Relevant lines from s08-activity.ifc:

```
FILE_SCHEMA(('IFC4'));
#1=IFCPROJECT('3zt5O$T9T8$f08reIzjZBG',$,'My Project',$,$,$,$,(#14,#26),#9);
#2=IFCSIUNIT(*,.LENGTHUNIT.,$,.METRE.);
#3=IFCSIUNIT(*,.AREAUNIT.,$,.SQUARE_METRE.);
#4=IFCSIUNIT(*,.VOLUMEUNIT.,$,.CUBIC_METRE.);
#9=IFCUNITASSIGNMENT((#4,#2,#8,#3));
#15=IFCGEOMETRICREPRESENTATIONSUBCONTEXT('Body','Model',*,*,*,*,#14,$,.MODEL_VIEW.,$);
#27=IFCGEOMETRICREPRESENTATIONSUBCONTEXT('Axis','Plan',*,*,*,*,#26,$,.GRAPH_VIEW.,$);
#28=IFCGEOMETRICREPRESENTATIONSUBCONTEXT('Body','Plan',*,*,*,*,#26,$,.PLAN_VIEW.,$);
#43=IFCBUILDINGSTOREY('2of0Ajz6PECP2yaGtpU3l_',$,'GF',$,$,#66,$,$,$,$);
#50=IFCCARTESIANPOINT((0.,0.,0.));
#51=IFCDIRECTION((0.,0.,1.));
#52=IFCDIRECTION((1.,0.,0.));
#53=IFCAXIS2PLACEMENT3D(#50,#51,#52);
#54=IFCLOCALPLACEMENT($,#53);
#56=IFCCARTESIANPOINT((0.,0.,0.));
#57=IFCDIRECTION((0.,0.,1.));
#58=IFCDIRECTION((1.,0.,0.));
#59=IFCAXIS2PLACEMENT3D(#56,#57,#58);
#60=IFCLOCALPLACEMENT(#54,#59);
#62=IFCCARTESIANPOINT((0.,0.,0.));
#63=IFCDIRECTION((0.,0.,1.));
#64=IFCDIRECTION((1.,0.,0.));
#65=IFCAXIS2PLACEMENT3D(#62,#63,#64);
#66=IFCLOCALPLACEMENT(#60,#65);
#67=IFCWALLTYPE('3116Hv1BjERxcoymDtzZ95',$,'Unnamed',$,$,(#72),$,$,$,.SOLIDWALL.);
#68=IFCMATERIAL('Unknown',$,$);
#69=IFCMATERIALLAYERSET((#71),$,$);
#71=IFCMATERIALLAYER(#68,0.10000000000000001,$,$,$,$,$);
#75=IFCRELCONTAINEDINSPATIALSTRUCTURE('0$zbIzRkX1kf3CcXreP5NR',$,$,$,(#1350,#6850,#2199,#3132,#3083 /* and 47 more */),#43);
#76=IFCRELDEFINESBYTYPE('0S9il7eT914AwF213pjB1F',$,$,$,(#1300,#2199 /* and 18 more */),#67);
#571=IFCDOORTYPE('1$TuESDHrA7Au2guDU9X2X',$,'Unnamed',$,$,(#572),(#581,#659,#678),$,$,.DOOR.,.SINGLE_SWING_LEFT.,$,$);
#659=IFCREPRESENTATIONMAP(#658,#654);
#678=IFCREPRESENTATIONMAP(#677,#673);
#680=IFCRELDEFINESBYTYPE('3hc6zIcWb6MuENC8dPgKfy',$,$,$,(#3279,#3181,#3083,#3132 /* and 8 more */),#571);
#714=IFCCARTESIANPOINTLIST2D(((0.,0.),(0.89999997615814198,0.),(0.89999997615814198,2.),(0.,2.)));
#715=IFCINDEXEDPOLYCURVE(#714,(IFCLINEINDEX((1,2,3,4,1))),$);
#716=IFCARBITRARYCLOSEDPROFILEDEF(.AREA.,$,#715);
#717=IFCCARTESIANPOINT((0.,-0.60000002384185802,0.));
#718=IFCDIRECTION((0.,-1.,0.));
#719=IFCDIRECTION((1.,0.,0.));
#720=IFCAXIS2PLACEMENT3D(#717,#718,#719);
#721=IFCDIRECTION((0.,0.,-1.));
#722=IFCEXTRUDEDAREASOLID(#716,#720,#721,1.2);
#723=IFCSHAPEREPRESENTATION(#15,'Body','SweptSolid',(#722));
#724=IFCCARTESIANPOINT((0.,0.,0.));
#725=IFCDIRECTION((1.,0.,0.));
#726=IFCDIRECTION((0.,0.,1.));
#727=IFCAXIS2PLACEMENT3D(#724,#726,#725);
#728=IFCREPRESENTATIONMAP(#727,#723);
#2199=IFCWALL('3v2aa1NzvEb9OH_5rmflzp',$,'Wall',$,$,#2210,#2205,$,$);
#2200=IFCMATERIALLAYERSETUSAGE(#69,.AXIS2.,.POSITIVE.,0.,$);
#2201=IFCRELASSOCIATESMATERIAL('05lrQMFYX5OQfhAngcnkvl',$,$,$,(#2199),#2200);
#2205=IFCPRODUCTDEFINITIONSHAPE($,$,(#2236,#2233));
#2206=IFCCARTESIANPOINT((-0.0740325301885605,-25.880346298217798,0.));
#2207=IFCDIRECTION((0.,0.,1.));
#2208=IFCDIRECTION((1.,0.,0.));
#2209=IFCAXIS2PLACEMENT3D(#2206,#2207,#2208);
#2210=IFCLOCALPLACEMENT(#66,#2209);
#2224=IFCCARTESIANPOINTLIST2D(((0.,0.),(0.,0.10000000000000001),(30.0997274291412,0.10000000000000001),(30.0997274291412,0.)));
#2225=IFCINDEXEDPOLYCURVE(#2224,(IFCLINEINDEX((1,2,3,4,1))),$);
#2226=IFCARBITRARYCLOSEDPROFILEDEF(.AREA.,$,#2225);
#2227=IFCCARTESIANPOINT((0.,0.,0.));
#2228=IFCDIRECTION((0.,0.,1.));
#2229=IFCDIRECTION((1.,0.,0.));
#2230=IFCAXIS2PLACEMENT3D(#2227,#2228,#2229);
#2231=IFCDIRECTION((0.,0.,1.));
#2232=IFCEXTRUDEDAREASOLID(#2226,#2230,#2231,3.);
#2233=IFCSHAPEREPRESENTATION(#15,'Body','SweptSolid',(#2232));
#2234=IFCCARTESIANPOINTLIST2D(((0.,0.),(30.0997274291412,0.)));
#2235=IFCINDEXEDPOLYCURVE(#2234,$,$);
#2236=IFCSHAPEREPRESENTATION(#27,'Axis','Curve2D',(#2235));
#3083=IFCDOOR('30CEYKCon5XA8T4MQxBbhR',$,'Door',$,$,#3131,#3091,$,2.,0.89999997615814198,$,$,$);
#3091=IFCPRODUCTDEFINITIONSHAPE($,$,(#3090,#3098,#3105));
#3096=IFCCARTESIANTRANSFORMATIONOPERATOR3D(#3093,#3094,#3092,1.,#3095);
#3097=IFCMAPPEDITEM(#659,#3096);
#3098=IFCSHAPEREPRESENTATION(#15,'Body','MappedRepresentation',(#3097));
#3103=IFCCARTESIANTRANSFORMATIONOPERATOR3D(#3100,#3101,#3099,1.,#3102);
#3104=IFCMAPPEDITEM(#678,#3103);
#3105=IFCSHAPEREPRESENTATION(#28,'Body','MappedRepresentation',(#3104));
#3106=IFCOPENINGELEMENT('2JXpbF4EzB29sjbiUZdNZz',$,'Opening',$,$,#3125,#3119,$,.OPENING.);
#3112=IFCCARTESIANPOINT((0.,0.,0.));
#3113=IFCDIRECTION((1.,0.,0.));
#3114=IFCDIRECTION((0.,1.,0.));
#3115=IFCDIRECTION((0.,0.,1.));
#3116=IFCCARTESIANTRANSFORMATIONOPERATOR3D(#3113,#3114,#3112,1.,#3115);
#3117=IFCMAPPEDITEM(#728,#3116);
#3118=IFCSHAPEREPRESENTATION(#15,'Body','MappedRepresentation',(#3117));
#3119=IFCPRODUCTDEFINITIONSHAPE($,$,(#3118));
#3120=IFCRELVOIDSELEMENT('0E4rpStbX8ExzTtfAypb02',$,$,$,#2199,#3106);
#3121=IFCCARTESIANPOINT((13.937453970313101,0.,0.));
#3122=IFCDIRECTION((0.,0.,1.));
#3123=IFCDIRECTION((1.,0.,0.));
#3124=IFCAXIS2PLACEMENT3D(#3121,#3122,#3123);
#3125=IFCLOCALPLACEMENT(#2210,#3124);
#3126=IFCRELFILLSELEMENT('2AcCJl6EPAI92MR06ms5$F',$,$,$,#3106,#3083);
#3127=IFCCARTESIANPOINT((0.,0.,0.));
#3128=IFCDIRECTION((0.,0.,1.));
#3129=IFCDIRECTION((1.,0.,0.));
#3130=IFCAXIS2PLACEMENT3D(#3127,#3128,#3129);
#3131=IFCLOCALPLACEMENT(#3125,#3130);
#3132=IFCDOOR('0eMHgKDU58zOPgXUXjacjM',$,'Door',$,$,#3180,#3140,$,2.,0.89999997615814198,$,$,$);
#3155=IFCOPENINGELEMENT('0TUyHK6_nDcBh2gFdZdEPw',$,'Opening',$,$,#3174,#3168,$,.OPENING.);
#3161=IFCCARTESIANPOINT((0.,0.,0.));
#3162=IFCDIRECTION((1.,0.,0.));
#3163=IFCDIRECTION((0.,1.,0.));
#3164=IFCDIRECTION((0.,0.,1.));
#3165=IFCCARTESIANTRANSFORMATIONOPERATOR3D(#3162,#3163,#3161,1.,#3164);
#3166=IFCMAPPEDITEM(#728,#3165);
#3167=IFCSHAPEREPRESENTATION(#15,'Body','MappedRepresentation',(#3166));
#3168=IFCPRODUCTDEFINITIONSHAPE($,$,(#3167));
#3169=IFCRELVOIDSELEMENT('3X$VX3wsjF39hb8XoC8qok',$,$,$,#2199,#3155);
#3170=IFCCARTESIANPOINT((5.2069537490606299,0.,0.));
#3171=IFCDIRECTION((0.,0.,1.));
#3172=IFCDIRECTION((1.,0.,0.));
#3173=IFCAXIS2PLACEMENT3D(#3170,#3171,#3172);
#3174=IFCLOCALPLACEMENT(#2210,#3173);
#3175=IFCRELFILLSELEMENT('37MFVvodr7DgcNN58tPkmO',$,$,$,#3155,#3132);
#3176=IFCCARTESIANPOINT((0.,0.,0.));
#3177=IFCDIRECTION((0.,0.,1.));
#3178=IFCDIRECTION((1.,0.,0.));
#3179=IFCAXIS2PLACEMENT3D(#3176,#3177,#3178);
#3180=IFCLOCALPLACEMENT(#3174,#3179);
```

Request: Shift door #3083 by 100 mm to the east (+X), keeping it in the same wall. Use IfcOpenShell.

```python
import ifcopenshell
import ifcopenshell.api.geometry
import ifcopenshell.util.placement

model = ifcopenshell.open("s08-activity.ifc")

door = model.by_guid("30CEYKCon5XA8T4MQxBbhR")
opening = door.FillsVoids[0].RelatingOpeningElement
wall = opening.VoidsElements[0].RelatingBuildingElement

wall_matrix = ifcopenshell.util.placement.get_local_placement(wall.ObjectPlacement)
shift = wall_matrix[:3, 0] * 0.1
before = ifcopenshell.util.placement.get_local_placement(door.ObjectPlacement)[:3, 3].copy()

# The door is placed relative to its opening, so it follows when the opening moves.
matrix = ifcopenshell.util.placement.get_local_placement(opening.ObjectPlacement)
matrix[:3, 3] += shift
ifcopenshell.api.geometry.edit_object_placement(
    model, product=opening, matrix=matrix, is_si=False, should_transform_children=True
)

after = ifcopenshell.util.placement.get_local_placement(door.ObjectPlacement)[:3, 3]
print("door moved by", (after - before).round(3) + 0.0)

model.write("s08-activity_updated.ifc")
```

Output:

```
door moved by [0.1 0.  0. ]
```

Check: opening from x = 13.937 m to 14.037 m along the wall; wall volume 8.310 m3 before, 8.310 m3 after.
